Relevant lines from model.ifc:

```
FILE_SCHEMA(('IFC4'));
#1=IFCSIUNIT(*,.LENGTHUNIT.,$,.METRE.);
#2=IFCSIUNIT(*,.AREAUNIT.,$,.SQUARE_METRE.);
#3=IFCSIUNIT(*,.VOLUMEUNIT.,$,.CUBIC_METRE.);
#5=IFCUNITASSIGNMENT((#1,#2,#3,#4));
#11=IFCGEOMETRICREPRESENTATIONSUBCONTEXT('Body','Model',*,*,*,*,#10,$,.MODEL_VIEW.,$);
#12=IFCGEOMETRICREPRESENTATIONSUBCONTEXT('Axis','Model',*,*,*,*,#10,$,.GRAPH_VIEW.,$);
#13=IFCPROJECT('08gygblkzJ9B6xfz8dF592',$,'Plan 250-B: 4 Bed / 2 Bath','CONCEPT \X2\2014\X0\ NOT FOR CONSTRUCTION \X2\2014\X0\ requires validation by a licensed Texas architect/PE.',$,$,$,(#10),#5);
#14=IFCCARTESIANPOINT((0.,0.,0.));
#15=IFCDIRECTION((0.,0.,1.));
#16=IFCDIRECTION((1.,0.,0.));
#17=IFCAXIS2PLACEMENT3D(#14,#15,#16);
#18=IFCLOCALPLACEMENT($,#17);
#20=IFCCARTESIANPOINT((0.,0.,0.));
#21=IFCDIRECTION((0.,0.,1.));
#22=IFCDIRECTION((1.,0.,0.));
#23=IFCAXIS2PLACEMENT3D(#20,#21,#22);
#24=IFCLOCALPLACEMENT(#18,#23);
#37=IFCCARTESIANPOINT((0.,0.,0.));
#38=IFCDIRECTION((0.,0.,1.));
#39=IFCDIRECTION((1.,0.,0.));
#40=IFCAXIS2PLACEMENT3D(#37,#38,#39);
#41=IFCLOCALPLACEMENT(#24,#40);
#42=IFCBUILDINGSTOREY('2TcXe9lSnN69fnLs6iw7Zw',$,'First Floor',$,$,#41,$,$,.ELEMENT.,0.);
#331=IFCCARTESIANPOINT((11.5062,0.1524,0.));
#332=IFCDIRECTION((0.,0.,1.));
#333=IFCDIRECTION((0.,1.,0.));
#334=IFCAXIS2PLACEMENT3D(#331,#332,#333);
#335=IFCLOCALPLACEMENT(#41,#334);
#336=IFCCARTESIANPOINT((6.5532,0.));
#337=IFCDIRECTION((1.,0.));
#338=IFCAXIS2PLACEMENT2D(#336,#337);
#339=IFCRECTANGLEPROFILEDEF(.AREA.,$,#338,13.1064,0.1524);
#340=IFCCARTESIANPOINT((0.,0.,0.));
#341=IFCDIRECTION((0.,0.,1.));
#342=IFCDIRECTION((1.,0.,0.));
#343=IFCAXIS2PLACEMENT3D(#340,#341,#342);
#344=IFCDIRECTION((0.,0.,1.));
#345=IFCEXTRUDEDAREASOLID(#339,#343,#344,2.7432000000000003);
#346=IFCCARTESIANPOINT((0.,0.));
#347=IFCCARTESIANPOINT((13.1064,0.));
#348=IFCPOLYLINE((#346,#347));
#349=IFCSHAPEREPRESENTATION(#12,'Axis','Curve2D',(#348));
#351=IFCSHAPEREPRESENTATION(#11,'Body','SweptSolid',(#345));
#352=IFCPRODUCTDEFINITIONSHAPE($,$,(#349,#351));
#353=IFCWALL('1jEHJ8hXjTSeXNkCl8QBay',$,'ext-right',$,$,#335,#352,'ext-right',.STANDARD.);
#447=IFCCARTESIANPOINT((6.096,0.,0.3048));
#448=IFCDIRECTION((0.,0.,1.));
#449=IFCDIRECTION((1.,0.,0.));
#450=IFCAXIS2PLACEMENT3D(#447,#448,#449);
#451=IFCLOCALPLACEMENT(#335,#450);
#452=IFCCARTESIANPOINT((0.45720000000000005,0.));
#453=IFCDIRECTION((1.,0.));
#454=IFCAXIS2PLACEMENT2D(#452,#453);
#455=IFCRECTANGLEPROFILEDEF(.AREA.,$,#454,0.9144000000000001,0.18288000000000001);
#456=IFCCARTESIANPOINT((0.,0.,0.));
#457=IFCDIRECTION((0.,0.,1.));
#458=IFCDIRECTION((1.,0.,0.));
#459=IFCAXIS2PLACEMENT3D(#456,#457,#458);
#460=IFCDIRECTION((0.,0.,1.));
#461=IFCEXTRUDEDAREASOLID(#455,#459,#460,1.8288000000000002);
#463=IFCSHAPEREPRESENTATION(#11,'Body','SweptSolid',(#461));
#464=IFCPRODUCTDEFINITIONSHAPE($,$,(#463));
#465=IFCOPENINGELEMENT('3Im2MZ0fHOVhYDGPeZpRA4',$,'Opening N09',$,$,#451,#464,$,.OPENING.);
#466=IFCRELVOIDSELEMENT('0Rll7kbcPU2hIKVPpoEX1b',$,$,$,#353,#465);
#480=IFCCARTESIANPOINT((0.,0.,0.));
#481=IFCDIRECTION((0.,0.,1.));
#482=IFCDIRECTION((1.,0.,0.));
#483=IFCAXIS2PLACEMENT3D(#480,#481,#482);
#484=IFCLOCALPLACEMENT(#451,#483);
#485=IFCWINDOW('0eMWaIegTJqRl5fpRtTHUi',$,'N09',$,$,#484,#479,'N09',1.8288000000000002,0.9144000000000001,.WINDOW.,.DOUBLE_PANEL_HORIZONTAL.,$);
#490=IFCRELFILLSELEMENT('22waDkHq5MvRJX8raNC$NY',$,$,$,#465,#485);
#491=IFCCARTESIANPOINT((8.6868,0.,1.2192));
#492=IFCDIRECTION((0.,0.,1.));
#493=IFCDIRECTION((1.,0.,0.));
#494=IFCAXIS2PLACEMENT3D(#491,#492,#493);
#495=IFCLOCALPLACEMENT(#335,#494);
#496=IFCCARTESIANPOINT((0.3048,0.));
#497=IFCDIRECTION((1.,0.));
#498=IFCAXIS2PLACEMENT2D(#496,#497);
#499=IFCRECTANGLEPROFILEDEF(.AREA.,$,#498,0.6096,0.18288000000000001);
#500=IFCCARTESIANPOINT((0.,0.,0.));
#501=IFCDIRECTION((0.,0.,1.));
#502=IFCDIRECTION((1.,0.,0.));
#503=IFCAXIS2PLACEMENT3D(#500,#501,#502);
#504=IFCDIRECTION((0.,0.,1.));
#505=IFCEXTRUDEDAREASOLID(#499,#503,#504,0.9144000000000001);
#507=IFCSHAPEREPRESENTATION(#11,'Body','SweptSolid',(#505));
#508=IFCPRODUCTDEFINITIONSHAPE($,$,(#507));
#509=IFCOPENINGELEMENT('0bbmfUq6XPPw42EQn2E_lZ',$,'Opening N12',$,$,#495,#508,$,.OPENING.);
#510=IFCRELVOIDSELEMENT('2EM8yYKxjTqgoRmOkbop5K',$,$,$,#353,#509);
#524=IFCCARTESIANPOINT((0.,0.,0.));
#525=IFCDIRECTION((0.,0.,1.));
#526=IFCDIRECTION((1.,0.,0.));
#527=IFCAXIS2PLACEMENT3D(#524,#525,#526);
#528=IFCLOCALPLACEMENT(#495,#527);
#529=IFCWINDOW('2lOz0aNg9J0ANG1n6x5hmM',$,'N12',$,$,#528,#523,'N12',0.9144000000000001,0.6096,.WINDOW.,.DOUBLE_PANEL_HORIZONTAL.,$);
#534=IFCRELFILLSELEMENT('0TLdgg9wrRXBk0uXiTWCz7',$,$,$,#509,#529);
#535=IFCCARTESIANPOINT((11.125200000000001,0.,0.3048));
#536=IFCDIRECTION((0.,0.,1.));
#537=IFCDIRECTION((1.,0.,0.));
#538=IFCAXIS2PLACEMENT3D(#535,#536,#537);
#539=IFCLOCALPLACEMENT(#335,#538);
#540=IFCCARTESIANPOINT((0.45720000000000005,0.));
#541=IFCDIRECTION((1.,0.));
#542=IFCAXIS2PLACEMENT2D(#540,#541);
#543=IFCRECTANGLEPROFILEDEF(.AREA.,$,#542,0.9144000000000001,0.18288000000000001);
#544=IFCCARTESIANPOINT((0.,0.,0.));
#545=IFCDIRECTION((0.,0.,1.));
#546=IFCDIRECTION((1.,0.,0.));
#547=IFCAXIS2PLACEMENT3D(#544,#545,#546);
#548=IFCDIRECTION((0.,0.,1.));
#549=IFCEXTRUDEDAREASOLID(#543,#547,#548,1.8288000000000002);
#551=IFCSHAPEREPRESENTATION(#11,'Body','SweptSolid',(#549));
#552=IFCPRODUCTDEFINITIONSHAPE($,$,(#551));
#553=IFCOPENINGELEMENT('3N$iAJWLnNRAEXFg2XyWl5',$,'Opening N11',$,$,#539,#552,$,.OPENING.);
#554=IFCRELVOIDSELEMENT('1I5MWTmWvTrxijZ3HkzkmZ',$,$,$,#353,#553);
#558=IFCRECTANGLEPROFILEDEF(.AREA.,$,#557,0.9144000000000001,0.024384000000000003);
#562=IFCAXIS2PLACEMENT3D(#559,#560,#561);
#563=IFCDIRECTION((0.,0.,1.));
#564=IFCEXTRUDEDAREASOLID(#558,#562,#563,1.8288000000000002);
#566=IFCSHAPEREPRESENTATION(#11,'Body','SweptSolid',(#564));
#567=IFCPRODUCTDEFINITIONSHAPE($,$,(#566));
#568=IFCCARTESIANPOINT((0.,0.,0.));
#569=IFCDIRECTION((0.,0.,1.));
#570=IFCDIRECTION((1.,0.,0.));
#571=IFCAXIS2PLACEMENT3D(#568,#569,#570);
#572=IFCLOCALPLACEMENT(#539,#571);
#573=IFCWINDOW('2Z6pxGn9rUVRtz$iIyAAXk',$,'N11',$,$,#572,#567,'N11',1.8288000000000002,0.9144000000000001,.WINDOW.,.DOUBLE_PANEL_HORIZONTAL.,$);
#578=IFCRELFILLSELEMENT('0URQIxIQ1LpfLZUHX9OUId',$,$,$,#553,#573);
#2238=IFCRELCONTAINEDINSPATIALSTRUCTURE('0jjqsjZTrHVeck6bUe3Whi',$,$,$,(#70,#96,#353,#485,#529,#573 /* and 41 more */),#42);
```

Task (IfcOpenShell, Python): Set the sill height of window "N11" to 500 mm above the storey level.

```python
import numpy as np
import ifcopenshell
import ifcopenshell.api.geometry
import ifcopenshell.geom
import ifcopenshell.util.element
import ifcopenshell.util.placement
import ifcopenshell.util.shape
import ifcopenshell.util.unit

model = ifcopenshell.open("model.ifc")
unit_scale = ifcopenshell.util.unit.calculate_unit_scale(model)

window = model.by_id(573)
opening = window.FillsVoids[0].RelatingOpeningElement
storey = ifcopenshell.util.element.get_container(window, ifc_class="IfcBuildingStorey")
level = ifcopenshell.util.placement.get_local_placement(storey.ObjectPlacement)[2, 3]

# The opening's origin need not be at the sill, so measure its lowest point.
shape = ifcopenshell.geom.create_shape(ifcopenshell.geom.settings(), opening)
bottom = ifcopenshell.util.shape.get_shape_bottom_elevation(shape, shape.geometry) / unit_scale
dz = level + 0.5 - bottom

shift = np.array([0.0, 0.0, dz])
# The window is placed relative to its opening, so it follows when the opening moves.
matrix = ifcopenshell.util.placement.get_local_placement(opening.ObjectPlacement)
matrix[:3, 3] += shift
ifcopenshell.api.geometry.edit_object_placement(
    model, product=opening, matrix=matrix, is_si=False, should_transform_children=True
)

print(f"moved by {dz * unit_scale:+.3f} m")

model.write("model_updated.ifc")
```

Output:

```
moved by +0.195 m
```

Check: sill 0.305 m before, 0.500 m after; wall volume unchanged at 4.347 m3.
